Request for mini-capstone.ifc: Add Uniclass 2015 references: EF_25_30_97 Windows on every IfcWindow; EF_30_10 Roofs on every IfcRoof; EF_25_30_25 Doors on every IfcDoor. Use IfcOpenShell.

First a look at what the model holds.

```python
import ifcopenshell

model = ifcopenshell.open("mini-capstone.ifc")
print(model.schema)
print("classifications:", [c.Name for c in model.by_type("IfcClassification")])
for ifc_class in ("IfcDoor", "IfcRoof", "IfcStair", "IfcWall", "IfcWindow"):
    print(ifc_class, len(model.by_type(ifc_class)))
```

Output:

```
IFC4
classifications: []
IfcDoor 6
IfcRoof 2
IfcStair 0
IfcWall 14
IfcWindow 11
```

```python
import ifcopenshell
import ifcopenshell.api.classification

model = ifcopenshell.open("mini-capstone.ifc")

system = ifcopenshell.api.classification.add_classification(model, classification="Uniclass 2015")

codes = {
    "IfcWindow": ("EF_25_30_97", "Windows"),
    "IfcRoof": ("EF_30_10", "Roofs"),
    "IfcDoor": ("EF_25_30_25", "Doors"),
}
for ifc_class, (code, name) in codes.items():
    products = model.by_type(ifc_class)
    ifcopenshell.api.classification.add_reference(
        model, products=products, classification=system, identification=code, name=name
    )
    print(code, len(products))

model.write("mini-capstone_updated.ifc")
```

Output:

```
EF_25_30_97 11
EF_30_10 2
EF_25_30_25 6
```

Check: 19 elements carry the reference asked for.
